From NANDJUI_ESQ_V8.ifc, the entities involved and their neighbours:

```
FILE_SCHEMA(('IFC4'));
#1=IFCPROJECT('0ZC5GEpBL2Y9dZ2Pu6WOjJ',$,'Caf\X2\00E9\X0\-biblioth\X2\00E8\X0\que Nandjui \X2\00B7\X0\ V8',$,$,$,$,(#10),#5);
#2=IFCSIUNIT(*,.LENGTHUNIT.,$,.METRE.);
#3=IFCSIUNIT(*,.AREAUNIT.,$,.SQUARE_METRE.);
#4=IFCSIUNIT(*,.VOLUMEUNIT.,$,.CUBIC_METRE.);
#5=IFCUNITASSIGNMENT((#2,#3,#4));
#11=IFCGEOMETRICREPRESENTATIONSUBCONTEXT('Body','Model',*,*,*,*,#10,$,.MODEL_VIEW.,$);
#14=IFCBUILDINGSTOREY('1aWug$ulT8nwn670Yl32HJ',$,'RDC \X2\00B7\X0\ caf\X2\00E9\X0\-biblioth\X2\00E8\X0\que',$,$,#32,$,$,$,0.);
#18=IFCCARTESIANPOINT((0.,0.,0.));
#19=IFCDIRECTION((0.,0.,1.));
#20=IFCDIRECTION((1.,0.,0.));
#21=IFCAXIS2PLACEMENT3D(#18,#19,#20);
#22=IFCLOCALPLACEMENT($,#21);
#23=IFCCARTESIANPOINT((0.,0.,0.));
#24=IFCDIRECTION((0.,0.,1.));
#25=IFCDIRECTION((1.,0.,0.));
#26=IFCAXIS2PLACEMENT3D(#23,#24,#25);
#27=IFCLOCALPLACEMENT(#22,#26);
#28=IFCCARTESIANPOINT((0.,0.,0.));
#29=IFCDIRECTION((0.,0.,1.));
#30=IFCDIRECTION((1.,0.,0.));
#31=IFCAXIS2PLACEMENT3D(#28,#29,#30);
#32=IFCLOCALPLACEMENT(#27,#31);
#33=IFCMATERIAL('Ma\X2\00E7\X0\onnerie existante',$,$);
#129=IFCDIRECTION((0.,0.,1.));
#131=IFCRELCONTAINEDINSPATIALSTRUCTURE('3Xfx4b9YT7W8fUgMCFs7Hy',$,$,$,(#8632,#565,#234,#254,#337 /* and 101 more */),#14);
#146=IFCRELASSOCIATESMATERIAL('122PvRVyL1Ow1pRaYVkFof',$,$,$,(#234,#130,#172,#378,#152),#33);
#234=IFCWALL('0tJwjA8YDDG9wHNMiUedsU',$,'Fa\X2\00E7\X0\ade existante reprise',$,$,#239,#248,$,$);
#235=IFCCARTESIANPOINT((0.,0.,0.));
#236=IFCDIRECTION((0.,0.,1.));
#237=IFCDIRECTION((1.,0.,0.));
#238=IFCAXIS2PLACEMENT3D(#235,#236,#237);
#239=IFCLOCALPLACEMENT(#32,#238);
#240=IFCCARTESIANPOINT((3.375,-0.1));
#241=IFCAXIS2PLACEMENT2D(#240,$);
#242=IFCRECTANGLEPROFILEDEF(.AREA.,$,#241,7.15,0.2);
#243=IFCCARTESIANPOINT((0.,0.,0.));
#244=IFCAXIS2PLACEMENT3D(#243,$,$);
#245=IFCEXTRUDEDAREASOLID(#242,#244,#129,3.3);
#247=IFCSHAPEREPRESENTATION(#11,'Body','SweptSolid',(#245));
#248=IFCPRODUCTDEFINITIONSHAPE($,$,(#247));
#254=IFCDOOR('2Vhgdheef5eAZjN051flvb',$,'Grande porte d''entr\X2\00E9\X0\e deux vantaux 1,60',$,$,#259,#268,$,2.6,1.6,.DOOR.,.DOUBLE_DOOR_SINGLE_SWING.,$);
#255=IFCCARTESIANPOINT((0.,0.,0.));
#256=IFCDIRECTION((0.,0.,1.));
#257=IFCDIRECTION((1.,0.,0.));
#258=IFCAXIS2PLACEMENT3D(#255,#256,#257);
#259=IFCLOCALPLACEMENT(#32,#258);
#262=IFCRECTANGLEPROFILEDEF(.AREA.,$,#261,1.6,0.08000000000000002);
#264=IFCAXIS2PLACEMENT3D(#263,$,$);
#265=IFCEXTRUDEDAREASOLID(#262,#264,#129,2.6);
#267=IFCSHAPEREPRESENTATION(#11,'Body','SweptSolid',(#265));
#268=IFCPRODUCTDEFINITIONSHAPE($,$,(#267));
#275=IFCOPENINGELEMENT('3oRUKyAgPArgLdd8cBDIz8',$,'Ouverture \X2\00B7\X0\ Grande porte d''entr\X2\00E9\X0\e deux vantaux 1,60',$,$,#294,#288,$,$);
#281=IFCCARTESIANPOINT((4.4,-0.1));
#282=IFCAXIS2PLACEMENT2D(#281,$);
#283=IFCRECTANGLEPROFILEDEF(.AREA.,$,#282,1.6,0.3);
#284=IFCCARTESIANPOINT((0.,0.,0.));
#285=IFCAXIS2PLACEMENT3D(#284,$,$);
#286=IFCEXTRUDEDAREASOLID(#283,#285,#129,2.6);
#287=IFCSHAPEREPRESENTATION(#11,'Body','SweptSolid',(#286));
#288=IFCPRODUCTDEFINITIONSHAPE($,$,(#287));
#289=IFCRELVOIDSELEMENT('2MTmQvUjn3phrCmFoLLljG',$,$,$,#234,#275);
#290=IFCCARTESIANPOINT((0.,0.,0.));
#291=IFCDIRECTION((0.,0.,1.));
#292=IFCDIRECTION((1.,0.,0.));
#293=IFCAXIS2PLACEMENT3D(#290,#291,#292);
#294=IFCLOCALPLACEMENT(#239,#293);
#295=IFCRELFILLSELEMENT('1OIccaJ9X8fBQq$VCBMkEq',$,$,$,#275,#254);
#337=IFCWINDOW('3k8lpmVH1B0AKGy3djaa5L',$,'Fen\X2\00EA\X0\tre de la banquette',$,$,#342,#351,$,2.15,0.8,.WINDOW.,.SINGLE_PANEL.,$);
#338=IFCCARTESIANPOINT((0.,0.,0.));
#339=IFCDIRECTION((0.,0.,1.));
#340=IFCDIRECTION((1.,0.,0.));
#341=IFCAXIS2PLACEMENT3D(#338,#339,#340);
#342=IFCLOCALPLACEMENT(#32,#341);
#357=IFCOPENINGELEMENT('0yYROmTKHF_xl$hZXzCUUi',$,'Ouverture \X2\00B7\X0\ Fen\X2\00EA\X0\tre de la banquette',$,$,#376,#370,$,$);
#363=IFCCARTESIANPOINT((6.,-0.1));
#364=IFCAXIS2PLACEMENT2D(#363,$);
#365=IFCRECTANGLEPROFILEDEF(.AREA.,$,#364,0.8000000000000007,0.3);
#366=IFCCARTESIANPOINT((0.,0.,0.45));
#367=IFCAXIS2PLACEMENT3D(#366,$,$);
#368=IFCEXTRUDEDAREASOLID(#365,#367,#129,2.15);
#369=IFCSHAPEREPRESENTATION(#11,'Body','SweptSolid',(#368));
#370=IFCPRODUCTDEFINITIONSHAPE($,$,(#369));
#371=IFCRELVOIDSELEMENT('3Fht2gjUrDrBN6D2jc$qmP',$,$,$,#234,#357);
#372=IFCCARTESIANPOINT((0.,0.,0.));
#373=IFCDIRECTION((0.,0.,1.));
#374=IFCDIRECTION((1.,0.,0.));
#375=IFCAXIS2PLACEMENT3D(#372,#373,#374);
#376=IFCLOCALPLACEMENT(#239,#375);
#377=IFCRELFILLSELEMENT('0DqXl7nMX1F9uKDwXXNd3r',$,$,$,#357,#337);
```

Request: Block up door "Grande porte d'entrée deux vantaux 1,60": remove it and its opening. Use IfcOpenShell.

```python
import ifcopenshell
import ifcopenshell.api.feature
import ifcopenshell.api.root
import ifcopenshell.geom
import ifcopenshell.util.shape

model = ifcopenshell.open("NANDJUI_ESQ_V8.ifc")
settings = ifcopenshell.geom.settings()


def volume(element):
    """Net volume in cubic metres, openings subtracted."""
    shape = ifcopenshell.geom.create_shape(settings, element)
    return ifcopenshell.util.shape.get_volume(shape.geometry)


door = model.by_guid("2Vhgdheef5eAZjN051flvb")
opening = door.FillsVoids[0].RelatingOpeningElement
wall = opening.VoidsElements[0].RelatingBuildingElement
before = volume(wall)

ifcopenshell.api.root.remove_product(model, product=door)
ifcopenshell.api.feature.remove_feature(model, feature=opening)

after = volume(wall)

print(f"wall volume {before:.3f} -> {after:.3f} m3")

model.write("NANDJUI_ESQ_V8_updated.ifc")
```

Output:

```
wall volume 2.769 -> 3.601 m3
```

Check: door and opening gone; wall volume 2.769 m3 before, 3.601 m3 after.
